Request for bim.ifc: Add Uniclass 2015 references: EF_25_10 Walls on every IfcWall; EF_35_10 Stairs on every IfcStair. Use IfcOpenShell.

First a look at what the model holds.

```python
import ifcopenshell

model = ifcopenshell.open("bim.ifc")
print(model.schema)
print("classifications:", [c.Name for c in model.by_type("IfcClassification")])
for ifc_class in ("IfcDoor", "IfcRoof", "IfcStair", "IfcWall", "IfcWindow"):
    print(ifc_class, len(model.by_type(ifc_class)))
```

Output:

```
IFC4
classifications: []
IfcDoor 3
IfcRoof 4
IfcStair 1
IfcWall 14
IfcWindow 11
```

```python
import ifcopenshell
import ifcopenshell.api.classification

model = ifcopenshell.open("bim.ifc")

system = ifcopenshell.api.classification.add_classification(model, classification="Uniclass 2015")

codes = {
    "IfcWall": ("EF_25_10", "Walls"),
    "IfcStair": ("EF_35_10", "Stairs"),
}
for ifc_class, (code, name) in codes.items():
    products = model.by_type(ifc_class)
    ifcopenshell.api.classification.add_reference(
        model, products=products, classification=system, identification=code, name=name
    )
    print(code, len(products))

model.write("bim_edited.ifc")
```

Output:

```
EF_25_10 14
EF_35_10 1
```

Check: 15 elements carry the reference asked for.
